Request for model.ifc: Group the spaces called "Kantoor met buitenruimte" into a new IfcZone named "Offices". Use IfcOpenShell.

First a look at what the model holds.

```python
import ifcopenshell

model = ifcopenshell.open("model.ifc")
print(model.schema)
seen = {}
for space in model.by_type("IfcSpace"):
    seen[space.LongName] = seen.get(space.LongName, 0) + 1
for name, count in sorted(seen.items(), key=str):
    print(count, "x", name)
print("zones:", [z.Name for z in model.by_type("IfcZone")][:20])
```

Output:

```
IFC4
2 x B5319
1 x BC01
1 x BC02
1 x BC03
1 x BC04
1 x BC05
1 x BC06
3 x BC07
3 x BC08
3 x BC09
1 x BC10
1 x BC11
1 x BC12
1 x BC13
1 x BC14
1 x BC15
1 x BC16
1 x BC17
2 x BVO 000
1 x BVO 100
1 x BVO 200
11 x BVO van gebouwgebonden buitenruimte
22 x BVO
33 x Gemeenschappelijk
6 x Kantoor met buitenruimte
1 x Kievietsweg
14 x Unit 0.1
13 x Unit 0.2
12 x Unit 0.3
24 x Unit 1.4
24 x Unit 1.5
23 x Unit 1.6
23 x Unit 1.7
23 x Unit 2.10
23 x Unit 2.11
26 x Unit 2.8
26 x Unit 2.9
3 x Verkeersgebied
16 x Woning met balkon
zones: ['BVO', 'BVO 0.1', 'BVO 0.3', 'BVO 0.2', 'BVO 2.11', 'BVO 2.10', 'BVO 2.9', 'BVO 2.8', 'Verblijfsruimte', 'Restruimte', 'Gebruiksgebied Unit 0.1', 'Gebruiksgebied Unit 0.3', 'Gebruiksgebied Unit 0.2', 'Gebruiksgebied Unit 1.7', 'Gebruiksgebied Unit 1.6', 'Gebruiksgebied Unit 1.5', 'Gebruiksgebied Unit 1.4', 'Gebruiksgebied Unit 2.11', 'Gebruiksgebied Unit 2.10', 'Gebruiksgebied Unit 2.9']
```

```python
import ifcopenshell
import ifcopenshell.api.group
import ifcopenshell.api.root

model = ifcopenshell.open("model.ifc")

names = {"Kantoor met buitenruimte"}
spaces = [s for s in model.by_type("IfcSpace") if s.LongName in names]

zone = ifcopenshell.api.root.create_entity(model, ifc_class="IfcZone", name="Offices")
ifcopenshell.api.group.assign_group(model, products=spaces, group=zone)
print(len(spaces), "spaces in", zone.Name)

model.write("model_rev.ifc")
```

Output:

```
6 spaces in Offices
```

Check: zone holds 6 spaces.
